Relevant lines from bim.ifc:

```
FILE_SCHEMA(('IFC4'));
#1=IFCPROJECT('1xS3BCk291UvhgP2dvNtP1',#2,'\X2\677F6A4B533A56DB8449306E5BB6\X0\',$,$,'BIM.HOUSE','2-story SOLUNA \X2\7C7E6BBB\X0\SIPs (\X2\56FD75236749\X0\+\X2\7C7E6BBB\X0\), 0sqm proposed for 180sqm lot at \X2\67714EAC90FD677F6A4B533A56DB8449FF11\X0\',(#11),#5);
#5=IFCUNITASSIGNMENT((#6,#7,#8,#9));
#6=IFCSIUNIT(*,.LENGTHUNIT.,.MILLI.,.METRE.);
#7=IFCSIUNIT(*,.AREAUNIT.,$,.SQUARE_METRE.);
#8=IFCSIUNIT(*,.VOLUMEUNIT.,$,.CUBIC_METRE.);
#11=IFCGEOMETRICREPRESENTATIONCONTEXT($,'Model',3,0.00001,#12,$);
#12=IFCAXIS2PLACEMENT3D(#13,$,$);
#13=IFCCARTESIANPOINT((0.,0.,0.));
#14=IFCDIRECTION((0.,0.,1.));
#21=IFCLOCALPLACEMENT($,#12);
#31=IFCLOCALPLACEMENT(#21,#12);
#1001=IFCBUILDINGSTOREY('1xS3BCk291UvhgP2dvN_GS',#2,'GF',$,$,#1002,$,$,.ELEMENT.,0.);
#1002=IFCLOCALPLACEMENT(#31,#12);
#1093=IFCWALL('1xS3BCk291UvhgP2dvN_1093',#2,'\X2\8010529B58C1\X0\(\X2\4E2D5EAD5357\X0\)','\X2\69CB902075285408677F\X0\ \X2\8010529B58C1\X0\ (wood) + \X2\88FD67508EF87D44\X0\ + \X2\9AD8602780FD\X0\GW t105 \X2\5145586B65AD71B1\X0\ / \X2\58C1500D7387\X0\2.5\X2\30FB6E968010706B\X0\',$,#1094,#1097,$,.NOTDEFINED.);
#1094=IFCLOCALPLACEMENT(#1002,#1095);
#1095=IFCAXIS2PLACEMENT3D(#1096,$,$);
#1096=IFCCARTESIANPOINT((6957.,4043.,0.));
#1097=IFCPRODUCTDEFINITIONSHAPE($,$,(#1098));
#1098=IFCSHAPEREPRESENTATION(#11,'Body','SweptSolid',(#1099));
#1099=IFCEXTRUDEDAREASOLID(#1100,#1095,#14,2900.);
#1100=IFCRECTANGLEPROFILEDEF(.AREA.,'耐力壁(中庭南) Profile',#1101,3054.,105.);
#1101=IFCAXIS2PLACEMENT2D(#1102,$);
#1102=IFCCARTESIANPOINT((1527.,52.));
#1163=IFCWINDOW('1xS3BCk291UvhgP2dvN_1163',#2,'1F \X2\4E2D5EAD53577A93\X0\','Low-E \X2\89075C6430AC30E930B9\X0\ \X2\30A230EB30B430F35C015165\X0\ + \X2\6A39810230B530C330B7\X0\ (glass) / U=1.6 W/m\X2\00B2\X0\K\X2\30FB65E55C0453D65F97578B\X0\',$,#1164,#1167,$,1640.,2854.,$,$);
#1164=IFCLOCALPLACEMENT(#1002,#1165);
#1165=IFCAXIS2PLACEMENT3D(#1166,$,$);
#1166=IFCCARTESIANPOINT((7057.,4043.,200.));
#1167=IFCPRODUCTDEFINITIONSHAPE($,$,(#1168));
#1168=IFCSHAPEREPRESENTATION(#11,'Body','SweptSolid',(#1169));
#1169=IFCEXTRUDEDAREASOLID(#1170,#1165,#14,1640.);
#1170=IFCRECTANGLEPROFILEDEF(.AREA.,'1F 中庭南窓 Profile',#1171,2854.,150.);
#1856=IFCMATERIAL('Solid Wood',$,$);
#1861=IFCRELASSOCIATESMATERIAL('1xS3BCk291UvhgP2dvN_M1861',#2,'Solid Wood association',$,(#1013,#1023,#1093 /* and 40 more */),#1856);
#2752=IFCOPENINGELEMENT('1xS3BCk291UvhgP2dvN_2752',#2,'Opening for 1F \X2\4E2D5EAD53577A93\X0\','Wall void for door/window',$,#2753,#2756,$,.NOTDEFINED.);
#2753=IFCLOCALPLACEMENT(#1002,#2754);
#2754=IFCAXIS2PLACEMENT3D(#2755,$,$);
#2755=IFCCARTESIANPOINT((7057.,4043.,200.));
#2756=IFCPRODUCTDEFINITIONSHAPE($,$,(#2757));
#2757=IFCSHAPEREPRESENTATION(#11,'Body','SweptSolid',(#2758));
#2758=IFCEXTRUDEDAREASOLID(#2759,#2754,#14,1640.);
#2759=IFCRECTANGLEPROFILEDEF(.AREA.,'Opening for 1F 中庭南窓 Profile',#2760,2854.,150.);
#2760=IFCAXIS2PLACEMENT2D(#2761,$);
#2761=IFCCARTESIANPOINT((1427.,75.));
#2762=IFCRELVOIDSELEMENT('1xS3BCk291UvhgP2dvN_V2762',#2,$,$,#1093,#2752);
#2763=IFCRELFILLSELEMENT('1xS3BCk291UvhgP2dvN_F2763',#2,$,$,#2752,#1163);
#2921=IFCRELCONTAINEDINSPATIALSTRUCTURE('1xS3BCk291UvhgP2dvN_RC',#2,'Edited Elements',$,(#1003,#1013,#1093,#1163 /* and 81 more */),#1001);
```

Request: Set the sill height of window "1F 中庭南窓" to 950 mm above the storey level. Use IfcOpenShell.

```python
import numpy as np
import ifcopenshell
import ifcopenshell.api.geometry
import ifcopenshell.geom
import ifcopenshell.util.element
import ifcopenshell.util.placement
import ifcopenshell.util.shape
import ifcopenshell.util.unit

model = ifcopenshell.open("bim.ifc")
unit_scale = ifcopenshell.util.unit.calculate_unit_scale(model)

window = model.by_guid("1xS3BCk291UvhgP2dvN_1163")
opening = window.FillsVoids[0].RelatingOpeningElement
storey = ifcopenshell.util.element.get_container(window, ifc_class="IfcBuildingStorey")
level = ifcopenshell.util.placement.get_local_placement(storey.ObjectPlacement)[2, 3]

# The opening's origin need not be at the sill, so measure its lowest point.
shape = ifcopenshell.geom.create_shape(ifcopenshell.geom.settings(), opening)
bottom = ifcopenshell.util.shape.get_shape_bottom_elevation(shape, shape.geometry) / unit_scale
dz = level + 0.95 / unit_scale - bottom

shift = np.array([0.0, 0.0, dz])
# The window is not placed relative to its opening, so move both.
for product in (opening, window):
    matrix = ifcopenshell.util.placement.get_local_placement(product.ObjectPlacement)
    matrix[:3, 3] += shift
    ifcopenshell.api.geometry.edit_object_placement(model, product=product, matrix=matrix, is_si=False)

print(f"moved by {dz * unit_scale:+.3f} m")

model.write("bim_updated.ifc")
```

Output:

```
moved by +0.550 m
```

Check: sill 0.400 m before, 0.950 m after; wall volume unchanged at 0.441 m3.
